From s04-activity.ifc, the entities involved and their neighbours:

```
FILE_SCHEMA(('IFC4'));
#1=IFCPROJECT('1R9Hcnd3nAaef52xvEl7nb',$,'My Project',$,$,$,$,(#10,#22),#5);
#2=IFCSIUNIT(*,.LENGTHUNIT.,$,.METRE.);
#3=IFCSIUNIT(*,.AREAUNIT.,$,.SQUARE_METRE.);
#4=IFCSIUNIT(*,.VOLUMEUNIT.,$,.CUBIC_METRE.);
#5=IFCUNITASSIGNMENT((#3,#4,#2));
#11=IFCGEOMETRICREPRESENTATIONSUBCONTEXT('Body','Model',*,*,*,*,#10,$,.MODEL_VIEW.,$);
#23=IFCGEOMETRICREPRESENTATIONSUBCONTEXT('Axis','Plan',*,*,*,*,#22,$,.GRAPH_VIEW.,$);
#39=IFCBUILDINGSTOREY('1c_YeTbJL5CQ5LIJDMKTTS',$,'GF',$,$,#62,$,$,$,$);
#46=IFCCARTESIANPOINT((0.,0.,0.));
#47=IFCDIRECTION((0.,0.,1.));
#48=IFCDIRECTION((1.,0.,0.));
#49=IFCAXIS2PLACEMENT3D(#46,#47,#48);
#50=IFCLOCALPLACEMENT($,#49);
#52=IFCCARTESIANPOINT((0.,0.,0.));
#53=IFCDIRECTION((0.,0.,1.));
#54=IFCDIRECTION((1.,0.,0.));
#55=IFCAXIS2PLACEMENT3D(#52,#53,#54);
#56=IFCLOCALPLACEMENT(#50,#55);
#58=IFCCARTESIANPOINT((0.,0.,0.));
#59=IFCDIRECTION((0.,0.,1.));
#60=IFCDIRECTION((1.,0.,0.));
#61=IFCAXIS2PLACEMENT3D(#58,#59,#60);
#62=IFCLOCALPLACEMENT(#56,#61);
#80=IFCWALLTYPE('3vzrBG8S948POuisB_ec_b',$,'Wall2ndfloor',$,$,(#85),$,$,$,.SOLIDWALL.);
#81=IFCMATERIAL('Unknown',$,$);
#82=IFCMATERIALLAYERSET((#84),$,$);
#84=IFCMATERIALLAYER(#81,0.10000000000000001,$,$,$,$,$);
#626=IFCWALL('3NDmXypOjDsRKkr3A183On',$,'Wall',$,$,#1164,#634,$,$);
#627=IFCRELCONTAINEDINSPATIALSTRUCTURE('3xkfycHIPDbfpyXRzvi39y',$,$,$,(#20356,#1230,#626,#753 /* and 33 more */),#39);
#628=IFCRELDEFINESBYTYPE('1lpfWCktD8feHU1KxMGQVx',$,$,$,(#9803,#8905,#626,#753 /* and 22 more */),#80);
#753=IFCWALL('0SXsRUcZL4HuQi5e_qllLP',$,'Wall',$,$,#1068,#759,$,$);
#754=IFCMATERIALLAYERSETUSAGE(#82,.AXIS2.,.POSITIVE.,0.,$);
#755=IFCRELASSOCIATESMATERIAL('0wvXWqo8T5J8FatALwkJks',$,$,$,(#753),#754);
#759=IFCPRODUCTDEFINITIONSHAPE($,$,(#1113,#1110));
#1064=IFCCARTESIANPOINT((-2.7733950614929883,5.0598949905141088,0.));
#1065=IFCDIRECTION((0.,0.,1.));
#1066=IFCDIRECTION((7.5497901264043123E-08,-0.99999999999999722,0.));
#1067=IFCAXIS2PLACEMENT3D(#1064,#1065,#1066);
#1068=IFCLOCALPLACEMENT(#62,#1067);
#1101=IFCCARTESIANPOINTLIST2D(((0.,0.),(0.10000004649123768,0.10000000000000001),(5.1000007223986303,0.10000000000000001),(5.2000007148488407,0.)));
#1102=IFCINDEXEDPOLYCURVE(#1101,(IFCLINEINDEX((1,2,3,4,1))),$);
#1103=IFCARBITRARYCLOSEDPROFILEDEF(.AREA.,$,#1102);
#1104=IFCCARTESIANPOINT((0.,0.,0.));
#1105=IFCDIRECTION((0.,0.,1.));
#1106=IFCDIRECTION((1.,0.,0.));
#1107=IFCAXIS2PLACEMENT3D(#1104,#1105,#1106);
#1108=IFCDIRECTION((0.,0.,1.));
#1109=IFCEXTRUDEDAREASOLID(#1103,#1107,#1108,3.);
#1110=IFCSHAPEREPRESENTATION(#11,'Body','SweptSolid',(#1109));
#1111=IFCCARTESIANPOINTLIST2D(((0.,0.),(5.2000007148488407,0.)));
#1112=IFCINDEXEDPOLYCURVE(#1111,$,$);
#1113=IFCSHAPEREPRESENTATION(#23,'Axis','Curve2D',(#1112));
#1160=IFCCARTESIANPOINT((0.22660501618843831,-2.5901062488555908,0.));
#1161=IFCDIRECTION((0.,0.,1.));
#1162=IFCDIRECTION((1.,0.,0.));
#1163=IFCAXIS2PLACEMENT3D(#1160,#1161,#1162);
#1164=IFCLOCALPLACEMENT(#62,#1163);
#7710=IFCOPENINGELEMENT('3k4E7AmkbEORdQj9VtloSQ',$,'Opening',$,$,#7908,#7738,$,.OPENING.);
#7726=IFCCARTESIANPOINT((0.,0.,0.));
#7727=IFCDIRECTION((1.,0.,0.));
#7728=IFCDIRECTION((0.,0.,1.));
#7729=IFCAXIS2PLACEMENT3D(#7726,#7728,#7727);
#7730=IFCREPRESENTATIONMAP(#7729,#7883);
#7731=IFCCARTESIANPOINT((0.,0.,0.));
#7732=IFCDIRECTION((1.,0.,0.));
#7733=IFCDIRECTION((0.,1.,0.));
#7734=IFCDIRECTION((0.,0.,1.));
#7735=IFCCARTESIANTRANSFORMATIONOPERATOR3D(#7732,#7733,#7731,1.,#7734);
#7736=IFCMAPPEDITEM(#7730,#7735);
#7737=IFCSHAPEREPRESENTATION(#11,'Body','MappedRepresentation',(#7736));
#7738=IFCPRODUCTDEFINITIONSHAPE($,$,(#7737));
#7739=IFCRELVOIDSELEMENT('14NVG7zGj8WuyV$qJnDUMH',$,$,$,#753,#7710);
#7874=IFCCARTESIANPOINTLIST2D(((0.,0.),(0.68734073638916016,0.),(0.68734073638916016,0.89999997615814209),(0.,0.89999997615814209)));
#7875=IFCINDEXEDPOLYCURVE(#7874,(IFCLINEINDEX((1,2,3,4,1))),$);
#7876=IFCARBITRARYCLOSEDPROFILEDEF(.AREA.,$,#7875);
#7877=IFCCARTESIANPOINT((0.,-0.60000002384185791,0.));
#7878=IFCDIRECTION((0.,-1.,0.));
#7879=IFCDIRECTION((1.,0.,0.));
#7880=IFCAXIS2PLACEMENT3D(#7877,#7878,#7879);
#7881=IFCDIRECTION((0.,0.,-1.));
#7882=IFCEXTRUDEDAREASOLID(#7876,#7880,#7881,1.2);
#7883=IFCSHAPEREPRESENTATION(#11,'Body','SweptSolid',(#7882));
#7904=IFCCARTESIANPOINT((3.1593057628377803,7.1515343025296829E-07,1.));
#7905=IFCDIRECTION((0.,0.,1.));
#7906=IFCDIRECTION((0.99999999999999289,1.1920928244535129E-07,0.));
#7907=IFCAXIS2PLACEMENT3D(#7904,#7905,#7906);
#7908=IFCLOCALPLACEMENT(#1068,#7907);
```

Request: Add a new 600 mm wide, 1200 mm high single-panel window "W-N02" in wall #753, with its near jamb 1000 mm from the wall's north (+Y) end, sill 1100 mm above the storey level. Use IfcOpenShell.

```python
import numpy as np
import ifcopenshell
import ifcopenshell.api.feature
import ifcopenshell.api.geometry
import ifcopenshell.api.root
import ifcopenshell.api.spatial
import ifcopenshell.geom
import ifcopenshell.util.element
import ifcopenshell.util.placement
import ifcopenshell.util.representation
import ifcopenshell.util.shape
import ifcopenshell.util.unit

model = ifcopenshell.open("s04-activity.ifc")
unit_scale = ifcopenshell.util.unit.calculate_unit_scale(model)
settings = ifcopenshell.geom.settings()


def volume(element):
    """Net volume in cubic metres, openings subtracted."""
    shape = ifcopenshell.geom.create_shape(settings, element)
    return ifcopenshell.util.shape.get_volume(shape.geometry)


wall = model.by_guid("0SXsRUcZL4HuQi5e_qllLP")
storey = ifcopenshell.util.element.get_container(wall, ifc_class="IfcBuildingStorey")
context = ifcopenshell.util.representation.get_context(model, "Model", "Body", "MODEL_VIEW")
before = volume(wall)

width, height, from_end, sill = 0.6, 1.2, 1, 1.1  # metres

# The wall runs along its own X axis, and the end named is its -X end.
wall_shape = ifcopenshell.geom.create_shape(settings, wall)
x, y, z = ifcopenshell.util.shape.get_vertices(wall_shape.geometry).T
start = x.min() + from_end
face, thickness = float(y.min()), float(y.max() - y.min())
wall_matrix = ifcopenshell.util.placement.get_local_placement(wall.ObjectPlacement)
level = ifcopenshell.util.placement.get_local_placement(storey.ObjectPlacement)[2, 3]


def in_wall(x, y):
    """Placement at x, y metres in the wall's axes, at sill height."""
    matrix = wall_matrix.copy()
    matrix[:, 3] = wall_matrix @ np.array([x / unit_scale, y / unit_scale, 0.0, 1.0])
    matrix[2, 3] = level + sill / unit_scale
    return matrix


# Opening: a box that overshoots both wall faces by 50 mm.
opening = ifcopenshell.api.root.create_entity(model, ifc_class="IfcOpeningElement", predefined_type="OPENING")
box = ifcopenshell.api.geometry.add_wall_representation(
    model, context=context, length=width, height=height, thickness=thickness + 0.1
)
ifcopenshell.api.geometry.assign_representation(model, product=opening, representation=box)
ifcopenshell.api.geometry.edit_object_placement(model, product=opening, matrix=in_wall(start, face - 0.05), is_si=False)
ifcopenshell.api.feature.add_feature(model, feature=opening, element=wall)

window = ifcopenshell.api.root.create_entity(model, ifc_class="IfcWindow", name="W-N02", predefined_type="WINDOW")
window.OverallWidth, window.OverallHeight = width / unit_scale, height / unit_scale
window.PartitioningType = "SINGLE_PANEL"
body = ifcopenshell.api.geometry.add_window_representation(
    model,
    context=context,
    overall_width=window.OverallWidth,
    overall_height=window.OverallHeight,
    partition_type="SINGLE_PANEL",
)
ifcopenshell.api.geometry.assign_representation(model, product=window, representation=body)
ifcopenshell.api.spatial.assign_container(model, products=[window], relating_structure=storey)
ifcopenshell.api.feature.add_filling(model, opening=opening, element=window)

# Centre the window in the wall's thickness.
ifcopenshell.api.geometry.edit_object_placement(model, product=window, matrix=in_wall(start, face), is_si=False)
window_shape = ifcopenshell.geom.create_shape(settings, window)
depth = ifcopenshell.util.shape.get_vertices(window_shape.geometry)[:, 1]
offset = face + thickness / 2 - (depth.min() + depth.max()) / 2
ifcopenshell.api.geometry.edit_object_placement(model, product=window, matrix=in_wall(start, offset), is_si=False)

after = volume(wall)

print(f"wall volume {before:.3f} -> {after:.3f} m3")

model.write("s04-activity-out.ifc")
```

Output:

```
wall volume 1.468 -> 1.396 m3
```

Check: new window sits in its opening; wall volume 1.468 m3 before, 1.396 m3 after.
